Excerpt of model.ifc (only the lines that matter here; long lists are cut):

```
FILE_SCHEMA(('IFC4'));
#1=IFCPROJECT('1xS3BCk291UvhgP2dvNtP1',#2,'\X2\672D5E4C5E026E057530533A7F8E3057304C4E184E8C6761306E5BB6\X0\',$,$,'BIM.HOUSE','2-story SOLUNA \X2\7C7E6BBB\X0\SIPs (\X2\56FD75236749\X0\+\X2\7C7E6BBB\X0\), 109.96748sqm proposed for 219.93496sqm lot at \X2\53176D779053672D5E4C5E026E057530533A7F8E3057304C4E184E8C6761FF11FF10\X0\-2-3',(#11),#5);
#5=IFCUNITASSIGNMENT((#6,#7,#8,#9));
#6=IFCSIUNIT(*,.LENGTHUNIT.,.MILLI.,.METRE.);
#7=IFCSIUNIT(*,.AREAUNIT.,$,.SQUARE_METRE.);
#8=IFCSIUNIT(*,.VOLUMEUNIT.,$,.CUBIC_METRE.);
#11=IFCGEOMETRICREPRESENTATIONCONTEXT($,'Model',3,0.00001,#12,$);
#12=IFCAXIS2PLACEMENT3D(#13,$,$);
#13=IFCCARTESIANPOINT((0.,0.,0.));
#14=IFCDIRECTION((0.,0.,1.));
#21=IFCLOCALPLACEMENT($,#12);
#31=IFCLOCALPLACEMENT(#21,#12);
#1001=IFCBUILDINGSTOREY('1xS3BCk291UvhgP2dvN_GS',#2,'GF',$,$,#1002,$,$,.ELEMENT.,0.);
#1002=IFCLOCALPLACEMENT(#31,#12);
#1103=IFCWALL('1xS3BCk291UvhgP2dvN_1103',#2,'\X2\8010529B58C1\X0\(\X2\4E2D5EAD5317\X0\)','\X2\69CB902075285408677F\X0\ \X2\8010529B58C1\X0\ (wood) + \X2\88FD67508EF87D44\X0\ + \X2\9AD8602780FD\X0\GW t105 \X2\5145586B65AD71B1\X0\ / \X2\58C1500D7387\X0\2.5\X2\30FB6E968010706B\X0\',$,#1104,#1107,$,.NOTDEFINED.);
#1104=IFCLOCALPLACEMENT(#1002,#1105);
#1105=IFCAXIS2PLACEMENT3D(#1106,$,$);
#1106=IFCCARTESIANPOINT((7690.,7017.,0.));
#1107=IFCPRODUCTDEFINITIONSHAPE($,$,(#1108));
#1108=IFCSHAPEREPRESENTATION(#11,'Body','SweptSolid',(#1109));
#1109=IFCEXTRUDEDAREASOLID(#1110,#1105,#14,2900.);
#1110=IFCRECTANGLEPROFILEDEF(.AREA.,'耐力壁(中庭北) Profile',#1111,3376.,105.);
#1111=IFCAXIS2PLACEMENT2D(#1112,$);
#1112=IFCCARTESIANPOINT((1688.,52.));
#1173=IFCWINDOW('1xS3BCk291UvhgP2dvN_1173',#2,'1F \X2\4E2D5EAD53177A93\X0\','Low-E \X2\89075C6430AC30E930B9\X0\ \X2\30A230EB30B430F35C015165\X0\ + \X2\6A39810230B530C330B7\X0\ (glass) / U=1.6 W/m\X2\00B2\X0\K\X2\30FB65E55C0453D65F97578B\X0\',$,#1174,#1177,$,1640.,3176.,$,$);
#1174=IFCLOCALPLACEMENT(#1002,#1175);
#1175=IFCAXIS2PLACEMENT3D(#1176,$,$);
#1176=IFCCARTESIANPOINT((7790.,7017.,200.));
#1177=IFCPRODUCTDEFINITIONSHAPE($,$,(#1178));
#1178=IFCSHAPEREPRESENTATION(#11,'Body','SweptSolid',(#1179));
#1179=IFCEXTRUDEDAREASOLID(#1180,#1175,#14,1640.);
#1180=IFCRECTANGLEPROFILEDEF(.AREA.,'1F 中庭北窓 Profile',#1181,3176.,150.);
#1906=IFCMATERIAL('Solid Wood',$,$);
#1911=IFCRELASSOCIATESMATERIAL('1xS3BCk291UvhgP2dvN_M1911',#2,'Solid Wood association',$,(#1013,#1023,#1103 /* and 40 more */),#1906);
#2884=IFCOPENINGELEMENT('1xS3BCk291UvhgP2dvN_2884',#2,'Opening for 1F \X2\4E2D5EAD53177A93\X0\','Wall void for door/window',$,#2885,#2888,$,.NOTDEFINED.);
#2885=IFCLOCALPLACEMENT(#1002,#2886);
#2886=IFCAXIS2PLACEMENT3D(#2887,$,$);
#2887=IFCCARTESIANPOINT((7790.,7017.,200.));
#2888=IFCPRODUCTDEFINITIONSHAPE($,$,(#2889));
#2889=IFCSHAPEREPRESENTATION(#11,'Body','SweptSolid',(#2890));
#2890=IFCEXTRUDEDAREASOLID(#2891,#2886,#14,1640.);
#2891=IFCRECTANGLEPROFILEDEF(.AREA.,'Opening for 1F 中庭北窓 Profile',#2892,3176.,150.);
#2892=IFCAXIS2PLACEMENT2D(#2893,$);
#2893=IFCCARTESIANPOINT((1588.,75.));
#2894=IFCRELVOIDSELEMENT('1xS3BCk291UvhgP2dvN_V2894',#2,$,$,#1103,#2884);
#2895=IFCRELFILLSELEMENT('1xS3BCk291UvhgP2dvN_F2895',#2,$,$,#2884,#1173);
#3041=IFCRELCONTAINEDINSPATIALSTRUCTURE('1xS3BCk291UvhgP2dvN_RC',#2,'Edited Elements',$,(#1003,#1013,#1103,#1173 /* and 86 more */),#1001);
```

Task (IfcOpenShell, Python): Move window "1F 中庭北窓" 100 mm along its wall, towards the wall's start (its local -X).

```python
import ifcopenshell
import ifcopenshell.api.geometry
import ifcopenshell.util.placement
import ifcopenshell.util.unit

model = ifcopenshell.open("model.ifc")
unit_scale = ifcopenshell.util.unit.calculate_unit_scale(model)

window = model.by_guid("1xS3BCk291UvhgP2dvN_1173")
opening = window.FillsVoids[0].RelatingOpeningElement
wall = opening.VoidsElements[0].RelatingBuildingElement

wall_matrix = ifcopenshell.util.placement.get_local_placement(wall.ObjectPlacement)
shift = wall_matrix[:3, 0] * -0.1 / unit_scale
before = ifcopenshell.util.placement.get_local_placement(window.ObjectPlacement)[:3, 3].copy()

# The window is not placed relative to its opening, so move both.
for product in (opening, window):
    matrix = ifcopenshell.util.placement.get_local_placement(product.ObjectPlacement)
    matrix[:3, 3] += shift
    ifcopenshell.api.geometry.edit_object_placement(model, product=product, matrix=matrix, is_si=False)

after = ifcopenshell.util.placement.get_local_placement(window.ObjectPlacement)[:3, 3]
print("window moved by", (after - before).round(3) + 0.0)

model.write("model_rev.ifc")
```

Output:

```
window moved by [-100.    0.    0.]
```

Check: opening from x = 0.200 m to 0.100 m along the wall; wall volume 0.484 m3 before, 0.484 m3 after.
